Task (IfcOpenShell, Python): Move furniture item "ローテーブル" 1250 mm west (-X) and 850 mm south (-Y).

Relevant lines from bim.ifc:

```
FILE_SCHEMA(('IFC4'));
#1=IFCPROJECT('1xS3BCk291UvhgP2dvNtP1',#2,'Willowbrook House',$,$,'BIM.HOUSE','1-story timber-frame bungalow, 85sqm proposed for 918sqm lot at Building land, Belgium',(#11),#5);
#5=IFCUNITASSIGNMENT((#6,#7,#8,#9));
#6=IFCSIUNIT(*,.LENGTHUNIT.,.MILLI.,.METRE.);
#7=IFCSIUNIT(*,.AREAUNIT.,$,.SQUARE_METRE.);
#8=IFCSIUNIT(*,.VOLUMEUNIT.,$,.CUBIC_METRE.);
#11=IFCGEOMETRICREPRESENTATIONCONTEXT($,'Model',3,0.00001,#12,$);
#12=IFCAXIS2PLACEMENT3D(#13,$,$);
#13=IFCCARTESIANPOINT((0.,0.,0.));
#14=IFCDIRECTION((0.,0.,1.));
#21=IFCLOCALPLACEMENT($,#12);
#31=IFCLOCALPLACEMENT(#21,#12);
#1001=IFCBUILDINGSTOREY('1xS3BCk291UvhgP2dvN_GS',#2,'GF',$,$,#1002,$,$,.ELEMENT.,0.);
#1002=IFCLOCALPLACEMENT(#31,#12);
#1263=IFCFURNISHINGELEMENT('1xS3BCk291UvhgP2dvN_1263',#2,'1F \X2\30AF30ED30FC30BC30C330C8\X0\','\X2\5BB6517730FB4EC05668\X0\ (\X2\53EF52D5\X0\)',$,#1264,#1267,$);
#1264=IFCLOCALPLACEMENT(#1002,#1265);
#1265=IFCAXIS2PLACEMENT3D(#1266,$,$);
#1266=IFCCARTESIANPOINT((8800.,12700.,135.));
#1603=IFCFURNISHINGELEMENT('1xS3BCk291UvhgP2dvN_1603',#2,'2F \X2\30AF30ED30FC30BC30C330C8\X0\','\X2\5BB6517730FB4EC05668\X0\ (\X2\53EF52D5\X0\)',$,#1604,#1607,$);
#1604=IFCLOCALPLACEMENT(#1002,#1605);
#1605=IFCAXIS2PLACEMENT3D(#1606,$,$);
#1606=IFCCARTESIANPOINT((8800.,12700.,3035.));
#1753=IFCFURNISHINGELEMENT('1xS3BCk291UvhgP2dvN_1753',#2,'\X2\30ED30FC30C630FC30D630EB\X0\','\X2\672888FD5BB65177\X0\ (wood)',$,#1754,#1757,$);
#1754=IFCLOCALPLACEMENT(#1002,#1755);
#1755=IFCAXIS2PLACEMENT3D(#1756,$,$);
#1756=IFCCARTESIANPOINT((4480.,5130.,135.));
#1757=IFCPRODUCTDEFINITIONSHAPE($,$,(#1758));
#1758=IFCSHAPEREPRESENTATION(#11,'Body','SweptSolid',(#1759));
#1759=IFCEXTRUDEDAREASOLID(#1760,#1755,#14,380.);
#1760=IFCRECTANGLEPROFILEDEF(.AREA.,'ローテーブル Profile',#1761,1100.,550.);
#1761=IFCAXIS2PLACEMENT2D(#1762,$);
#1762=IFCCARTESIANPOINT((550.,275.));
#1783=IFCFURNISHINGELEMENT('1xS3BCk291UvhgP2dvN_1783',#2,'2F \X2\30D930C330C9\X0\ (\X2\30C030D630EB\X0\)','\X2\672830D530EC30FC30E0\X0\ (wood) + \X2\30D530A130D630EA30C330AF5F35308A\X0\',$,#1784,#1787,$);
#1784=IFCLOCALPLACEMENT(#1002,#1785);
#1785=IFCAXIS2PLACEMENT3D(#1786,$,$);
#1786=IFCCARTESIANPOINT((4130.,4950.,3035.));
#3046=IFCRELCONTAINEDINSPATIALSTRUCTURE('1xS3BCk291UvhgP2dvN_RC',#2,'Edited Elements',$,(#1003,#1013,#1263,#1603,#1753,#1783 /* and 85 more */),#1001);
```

```python
import ifcopenshell
import ifcopenshell.api.geometry
import ifcopenshell.util.placement
import ifcopenshell.util.unit

model = ifcopenshell.open("bim.ifc")
unit_scale = ifcopenshell.util.unit.calculate_unit_scale(model)

item = model.by_guid("1xS3BCk291UvhgP2dvN_1753")
matrix = ifcopenshell.util.placement.get_local_placement(item.ObjectPlacement)
matrix[0, 3] -= 1.25 / unit_scale
matrix[1, 3] -= 0.85 / unit_scale
ifcopenshell.api.geometry.edit_object_placement(model, product=item, matrix=matrix, is_si=False)

print(ifcopenshell.util.placement.get_local_placement(item.ObjectPlacement).round(3) + 0.0)

model.write("bim_edited.ifc")
```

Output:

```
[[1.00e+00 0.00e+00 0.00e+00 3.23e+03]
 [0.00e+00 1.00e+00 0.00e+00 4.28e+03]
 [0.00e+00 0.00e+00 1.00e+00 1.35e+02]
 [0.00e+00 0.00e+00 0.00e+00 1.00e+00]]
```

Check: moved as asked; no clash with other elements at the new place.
